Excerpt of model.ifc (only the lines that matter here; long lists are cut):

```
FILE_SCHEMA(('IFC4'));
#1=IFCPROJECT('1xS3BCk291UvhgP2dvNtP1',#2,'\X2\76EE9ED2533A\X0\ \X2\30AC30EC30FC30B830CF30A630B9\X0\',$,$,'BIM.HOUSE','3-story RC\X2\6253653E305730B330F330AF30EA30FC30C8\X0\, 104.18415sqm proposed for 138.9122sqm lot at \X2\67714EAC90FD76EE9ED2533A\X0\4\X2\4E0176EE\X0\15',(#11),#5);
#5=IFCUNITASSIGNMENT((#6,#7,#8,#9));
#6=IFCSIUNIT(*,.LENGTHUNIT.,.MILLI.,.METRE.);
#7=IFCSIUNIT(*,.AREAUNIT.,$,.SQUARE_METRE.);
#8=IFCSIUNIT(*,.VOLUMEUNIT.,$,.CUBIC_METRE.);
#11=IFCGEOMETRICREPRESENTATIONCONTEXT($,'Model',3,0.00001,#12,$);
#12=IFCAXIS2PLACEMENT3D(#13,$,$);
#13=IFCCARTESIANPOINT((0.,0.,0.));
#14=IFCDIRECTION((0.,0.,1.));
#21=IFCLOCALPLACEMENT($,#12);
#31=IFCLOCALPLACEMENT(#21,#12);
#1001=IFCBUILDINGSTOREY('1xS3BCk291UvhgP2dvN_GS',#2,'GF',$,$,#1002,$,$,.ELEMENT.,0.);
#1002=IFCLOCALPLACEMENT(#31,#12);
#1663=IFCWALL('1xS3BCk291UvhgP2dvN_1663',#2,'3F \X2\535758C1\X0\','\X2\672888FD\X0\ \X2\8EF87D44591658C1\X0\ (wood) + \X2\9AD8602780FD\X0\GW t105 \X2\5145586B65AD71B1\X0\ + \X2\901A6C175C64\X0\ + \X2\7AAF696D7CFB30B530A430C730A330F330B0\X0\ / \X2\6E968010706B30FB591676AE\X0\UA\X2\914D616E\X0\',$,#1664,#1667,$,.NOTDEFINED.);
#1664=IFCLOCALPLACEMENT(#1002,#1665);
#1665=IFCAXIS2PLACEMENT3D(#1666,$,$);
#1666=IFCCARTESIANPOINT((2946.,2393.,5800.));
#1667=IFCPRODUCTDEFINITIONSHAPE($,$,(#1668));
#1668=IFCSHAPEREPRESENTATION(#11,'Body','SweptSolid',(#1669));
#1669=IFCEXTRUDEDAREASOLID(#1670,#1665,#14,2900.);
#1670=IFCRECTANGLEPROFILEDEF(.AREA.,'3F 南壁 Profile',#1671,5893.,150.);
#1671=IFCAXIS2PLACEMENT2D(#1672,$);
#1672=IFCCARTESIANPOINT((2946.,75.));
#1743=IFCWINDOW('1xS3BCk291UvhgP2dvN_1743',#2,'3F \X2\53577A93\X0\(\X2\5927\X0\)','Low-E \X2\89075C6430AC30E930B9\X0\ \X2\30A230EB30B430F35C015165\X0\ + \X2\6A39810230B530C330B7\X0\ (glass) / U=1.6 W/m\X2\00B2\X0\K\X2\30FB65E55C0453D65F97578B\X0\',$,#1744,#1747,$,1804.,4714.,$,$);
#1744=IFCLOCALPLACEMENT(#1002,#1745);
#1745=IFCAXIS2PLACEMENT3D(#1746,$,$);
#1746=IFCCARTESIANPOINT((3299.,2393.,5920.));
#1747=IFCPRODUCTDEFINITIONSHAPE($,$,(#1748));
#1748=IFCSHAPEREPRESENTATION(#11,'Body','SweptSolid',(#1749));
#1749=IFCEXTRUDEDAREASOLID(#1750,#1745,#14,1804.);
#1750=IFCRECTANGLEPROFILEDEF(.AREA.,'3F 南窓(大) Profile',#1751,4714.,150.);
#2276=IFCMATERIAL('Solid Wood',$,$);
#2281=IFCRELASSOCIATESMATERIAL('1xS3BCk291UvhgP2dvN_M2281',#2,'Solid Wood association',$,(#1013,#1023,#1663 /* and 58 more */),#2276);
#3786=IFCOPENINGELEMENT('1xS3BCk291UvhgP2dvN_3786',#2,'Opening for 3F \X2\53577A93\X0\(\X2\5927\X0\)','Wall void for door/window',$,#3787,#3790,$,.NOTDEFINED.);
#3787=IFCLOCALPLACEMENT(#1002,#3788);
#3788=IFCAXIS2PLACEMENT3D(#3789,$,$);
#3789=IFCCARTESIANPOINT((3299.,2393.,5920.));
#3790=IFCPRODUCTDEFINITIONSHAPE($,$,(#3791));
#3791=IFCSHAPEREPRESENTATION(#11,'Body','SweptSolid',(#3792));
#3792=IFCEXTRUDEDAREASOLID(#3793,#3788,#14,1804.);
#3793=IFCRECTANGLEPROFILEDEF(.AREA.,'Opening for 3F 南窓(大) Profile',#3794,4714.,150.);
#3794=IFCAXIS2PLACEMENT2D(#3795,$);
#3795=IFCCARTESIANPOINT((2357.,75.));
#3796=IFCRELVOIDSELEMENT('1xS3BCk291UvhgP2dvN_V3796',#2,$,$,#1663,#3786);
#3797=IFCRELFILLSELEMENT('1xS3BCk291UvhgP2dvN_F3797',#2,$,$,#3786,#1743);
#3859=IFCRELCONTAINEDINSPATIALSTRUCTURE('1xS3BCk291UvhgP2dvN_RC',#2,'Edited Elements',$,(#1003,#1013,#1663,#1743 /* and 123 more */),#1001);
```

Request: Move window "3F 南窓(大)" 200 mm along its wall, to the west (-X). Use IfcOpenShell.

```python
import ifcopenshell
import ifcopenshell.api.geometry
import ifcopenshell.util.placement

model = ifcopenshell.open("model.ifc")

window = model.by_id(1743)
opening = window.FillsVoids[0].RelatingOpeningElement
wall = opening.VoidsElements[0].RelatingBuildingElement

wall_matrix = ifcopenshell.util.placement.get_local_placement(wall.ObjectPlacement)
shift = wall_matrix[:3, 0] * -200.0
before = ifcopenshell.util.placement.get_local_placement(window.ObjectPlacement)[:3, 3].copy()

# The window is not placed relative to its opening, so move both.
for product in (opening, window):
    matrix = ifcopenshell.util.placement.get_local_placement(product.ObjectPlacement)
    matrix[:3, 3] += shift
    ifcopenshell.api.geometry.edit_object_placement(model, product=product, matrix=matrix, is_si=False)

after = ifcopenshell.util.placement.get_local_placement(window.ObjectPlacement)[:3, 3]
print("window moved by", (after - before).round(3) + 0.0)

model.write("model_updated.ifc")
```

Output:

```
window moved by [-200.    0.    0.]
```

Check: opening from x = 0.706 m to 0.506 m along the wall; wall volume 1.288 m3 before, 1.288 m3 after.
